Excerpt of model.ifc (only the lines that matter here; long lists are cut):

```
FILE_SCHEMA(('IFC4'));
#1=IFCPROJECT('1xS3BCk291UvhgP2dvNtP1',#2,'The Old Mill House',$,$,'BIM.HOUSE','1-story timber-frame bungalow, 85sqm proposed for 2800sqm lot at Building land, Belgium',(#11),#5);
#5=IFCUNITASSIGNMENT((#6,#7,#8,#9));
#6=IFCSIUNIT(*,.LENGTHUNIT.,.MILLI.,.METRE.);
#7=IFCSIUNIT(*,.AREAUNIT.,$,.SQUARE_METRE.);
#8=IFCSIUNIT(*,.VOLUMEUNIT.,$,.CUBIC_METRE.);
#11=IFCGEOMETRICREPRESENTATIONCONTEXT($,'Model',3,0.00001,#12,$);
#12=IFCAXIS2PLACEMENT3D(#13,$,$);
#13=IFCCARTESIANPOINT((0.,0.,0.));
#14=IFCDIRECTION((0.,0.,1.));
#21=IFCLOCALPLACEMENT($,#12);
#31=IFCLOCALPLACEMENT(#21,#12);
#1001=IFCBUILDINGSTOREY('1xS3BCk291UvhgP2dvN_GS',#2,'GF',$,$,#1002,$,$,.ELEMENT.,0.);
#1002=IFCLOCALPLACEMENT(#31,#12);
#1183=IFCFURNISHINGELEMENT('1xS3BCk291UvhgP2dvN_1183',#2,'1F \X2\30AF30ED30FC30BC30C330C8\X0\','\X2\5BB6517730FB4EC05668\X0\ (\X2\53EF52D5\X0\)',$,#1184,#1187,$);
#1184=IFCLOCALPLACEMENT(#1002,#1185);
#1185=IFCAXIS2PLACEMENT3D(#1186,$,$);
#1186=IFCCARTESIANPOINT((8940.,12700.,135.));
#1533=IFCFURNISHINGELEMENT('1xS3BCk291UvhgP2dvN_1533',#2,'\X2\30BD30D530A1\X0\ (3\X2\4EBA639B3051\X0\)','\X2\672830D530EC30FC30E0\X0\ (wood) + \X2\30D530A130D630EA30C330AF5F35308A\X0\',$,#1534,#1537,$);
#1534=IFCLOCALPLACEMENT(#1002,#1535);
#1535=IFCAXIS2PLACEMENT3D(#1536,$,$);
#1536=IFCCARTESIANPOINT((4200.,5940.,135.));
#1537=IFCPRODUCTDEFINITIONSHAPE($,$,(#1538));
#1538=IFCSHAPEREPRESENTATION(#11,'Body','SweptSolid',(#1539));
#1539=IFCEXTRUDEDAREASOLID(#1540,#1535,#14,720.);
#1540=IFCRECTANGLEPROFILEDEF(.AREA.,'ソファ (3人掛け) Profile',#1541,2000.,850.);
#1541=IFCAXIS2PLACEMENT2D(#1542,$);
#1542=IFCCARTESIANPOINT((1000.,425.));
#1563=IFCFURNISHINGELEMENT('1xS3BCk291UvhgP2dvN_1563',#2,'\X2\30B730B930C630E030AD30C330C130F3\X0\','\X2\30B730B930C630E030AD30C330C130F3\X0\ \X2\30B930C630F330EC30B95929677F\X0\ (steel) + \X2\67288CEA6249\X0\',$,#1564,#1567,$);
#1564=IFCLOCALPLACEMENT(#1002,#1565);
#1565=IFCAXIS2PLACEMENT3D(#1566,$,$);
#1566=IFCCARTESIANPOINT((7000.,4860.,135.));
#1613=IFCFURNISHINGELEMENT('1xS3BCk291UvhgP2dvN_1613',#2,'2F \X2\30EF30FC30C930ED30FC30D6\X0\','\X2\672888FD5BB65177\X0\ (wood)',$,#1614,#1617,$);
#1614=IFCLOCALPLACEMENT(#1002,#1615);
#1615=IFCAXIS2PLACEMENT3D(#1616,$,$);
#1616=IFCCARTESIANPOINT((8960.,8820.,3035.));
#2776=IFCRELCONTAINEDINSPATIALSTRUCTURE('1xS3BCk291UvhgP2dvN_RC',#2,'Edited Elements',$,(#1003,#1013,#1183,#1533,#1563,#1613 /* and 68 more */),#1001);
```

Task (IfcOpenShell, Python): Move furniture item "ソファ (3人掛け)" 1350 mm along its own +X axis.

```python
import ifcopenshell
import ifcopenshell.api.geometry
import ifcopenshell.util.placement

model = ifcopenshell.open("model.ifc")

item = model.by_guid("1xS3BCk291UvhgP2dvN_1533")
matrix = ifcopenshell.util.placement.get_local_placement(item.ObjectPlacement)
matrix[:3, 3] += matrix[:3, 0] * 1350.0
ifcopenshell.api.geometry.edit_object_placement(model, product=item, matrix=matrix, is_si=False)

print(ifcopenshell.util.placement.get_local_placement(item.ObjectPlacement).round(3) + 0.0)

model.write("model_v2.ifc")
```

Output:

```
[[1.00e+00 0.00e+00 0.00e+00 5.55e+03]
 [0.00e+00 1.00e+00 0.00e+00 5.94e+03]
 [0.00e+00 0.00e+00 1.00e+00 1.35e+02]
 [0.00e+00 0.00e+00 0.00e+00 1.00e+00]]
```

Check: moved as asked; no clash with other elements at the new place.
